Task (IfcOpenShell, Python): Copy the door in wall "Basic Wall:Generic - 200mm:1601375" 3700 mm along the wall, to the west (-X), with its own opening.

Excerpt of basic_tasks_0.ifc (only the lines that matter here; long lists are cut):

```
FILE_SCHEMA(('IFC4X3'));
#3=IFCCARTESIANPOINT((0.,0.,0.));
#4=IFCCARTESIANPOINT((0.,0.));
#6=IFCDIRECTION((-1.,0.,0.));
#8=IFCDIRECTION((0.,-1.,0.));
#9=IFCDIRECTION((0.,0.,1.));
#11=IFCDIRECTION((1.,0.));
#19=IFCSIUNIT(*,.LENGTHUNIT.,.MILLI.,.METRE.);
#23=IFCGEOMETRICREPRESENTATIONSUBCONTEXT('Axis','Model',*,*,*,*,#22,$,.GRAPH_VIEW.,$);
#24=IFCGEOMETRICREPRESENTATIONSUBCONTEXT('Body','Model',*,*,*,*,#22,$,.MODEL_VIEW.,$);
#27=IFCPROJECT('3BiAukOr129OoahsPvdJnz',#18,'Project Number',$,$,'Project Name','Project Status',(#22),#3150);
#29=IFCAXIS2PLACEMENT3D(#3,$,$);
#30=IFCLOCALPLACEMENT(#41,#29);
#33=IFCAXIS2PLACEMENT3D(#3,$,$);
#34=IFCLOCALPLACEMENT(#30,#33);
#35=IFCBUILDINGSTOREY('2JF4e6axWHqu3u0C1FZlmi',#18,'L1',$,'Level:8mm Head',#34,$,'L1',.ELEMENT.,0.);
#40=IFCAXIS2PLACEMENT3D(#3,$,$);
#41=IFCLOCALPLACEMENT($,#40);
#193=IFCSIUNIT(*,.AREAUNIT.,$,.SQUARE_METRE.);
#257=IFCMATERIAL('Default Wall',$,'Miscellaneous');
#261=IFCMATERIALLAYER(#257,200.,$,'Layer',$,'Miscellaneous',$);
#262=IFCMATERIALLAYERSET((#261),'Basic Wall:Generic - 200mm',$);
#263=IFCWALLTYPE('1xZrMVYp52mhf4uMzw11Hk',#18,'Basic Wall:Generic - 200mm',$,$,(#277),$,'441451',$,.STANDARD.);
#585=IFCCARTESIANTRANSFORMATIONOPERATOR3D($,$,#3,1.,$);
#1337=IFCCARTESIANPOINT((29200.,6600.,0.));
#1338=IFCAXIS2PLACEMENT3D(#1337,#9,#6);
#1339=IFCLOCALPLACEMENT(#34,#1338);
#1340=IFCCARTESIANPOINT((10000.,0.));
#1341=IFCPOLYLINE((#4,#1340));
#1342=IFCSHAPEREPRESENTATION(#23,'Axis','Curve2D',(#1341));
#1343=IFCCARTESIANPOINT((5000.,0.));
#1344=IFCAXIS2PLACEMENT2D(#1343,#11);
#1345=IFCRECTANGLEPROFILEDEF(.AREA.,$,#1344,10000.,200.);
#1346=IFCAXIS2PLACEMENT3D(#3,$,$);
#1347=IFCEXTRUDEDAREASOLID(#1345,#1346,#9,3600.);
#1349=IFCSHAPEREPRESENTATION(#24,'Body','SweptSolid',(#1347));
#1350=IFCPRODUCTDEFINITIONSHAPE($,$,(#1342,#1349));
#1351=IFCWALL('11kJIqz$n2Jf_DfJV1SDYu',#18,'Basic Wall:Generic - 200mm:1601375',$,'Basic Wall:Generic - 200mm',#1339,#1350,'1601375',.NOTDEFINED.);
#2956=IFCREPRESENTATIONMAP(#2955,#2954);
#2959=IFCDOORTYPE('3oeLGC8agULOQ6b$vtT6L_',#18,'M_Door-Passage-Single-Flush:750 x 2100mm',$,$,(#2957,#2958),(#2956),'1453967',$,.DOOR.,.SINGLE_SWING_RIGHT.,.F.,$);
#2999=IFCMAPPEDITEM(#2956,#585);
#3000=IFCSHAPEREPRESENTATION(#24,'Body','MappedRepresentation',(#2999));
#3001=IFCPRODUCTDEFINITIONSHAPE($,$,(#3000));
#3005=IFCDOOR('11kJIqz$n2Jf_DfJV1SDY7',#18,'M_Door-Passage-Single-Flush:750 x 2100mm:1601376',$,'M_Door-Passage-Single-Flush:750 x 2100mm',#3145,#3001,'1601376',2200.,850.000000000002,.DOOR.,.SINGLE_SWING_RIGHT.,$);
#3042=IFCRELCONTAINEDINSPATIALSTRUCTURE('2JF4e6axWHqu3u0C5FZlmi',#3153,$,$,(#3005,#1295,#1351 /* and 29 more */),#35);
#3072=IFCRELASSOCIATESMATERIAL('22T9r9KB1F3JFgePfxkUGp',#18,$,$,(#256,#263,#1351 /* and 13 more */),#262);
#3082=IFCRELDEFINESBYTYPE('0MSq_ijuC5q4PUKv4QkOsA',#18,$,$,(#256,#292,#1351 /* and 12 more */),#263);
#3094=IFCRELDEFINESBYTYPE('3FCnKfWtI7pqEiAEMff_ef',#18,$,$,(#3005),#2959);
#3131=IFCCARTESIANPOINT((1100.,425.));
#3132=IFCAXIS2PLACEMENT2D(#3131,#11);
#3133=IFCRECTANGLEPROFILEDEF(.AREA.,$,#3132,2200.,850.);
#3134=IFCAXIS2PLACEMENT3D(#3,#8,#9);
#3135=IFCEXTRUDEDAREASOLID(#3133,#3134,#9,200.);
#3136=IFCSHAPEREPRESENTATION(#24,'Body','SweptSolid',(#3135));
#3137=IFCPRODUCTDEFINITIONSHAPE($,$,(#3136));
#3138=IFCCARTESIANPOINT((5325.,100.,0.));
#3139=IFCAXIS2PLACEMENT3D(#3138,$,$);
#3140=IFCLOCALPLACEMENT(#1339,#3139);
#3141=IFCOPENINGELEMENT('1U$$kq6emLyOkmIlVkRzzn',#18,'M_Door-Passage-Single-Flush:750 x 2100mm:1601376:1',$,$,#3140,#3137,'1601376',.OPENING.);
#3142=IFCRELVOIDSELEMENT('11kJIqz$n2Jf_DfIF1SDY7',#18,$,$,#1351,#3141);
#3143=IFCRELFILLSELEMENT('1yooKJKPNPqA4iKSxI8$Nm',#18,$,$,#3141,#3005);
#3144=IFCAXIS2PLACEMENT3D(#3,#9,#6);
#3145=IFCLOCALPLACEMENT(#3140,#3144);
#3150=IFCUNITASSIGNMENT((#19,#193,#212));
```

```python
import ifcopenshell
import ifcopenshell.api.feature
import ifcopenshell.api.geometry
import ifcopenshell.api.root
import ifcopenshell.geom
import ifcopenshell.util.element
import ifcopenshell.util.placement
import ifcopenshell.util.shape

model = ifcopenshell.open("basic_tasks_0.ifc")
settings = ifcopenshell.geom.settings()


def volume(element):
    """Net volume in cubic metres, openings subtracted."""
    shape = ifcopenshell.geom.create_shape(settings, element)
    return ifcopenshell.util.shape.get_volume(shape.geometry)


def reuse_history(source, copy):
    """copy_class also copies each property set's owner history, people and application; keep the originals."""
    for rel in copy.IsDefinedBy:
        if rel.is_a("IfcRelDefinesByProperties") and (history := rel.RelatingPropertyDefinition.OwnerHistory):
            rel.RelatingPropertyDefinition.OwnerHistory = source.OwnerHistory
            ifcopenshell.util.element.remove_deep2(model, history)


door = model.by_guid("11kJIqz$n2Jf_DfJV1SDY7")
opening = door.FillsVoids[0].RelatingOpeningElement
wall = opening.VoidsElements[0].RelatingBuildingElement
before = volume(wall)
shift = ifcopenshell.util.placement.get_local_placement(wall.ObjectPlacement)[:3, 0] * 3700.0

# copy_class copies the void relationship, type, container and properties, but no geometry.
new_opening = ifcopenshell.api.root.copy_class(model, product=opening)
new_opening.Representation = ifcopenshell.util.element.copy_deep(
    model, opening.Representation, exclude=["IfcGeometricRepresentationContext", "IfcRepresentationMap"]
)
new_opening.Name = "M_Door-Passage-Single-Flush:750 x 2100mm"
new_opening.Tag = None
new_door = ifcopenshell.api.root.copy_class(model, product=door)
new_door.Representation = ifcopenshell.util.element.copy_deep(
    model, door.Representation, exclude=["IfcGeometricRepresentationContext", "IfcRepresentationMap"]
)
new_door.Name = "M_Door-Passage-Single-Flush:750 x 2100mm"
new_door.Tag = None
reuse_history(door, new_door)
ifcopenshell.api.feature.add_filling(model, opening=new_opening, element=new_door)

for old, new in ((opening, new_opening), (door, new_door)):
    matrix = ifcopenshell.util.placement.get_local_placement(old.ObjectPlacement)
    matrix[:3, 3] += shift
    ifcopenshell.api.geometry.edit_object_placement(model, product=new, matrix=matrix, is_si=False)

after = volume(wall)

print(f"wall volume {before:.3f} -> {after:.3f} m3")

model.write("basic_tasks_0_rev.ifc")
```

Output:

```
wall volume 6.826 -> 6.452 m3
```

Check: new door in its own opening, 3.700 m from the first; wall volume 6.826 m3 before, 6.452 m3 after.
